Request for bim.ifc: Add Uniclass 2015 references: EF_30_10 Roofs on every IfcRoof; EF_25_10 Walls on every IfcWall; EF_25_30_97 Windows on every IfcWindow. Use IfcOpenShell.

First a look at what the model holds.

```python
import ifcopenshell

model = ifcopenshell.open("bim.ifc")
print(model.schema)
print("classifications:", [c.Name for c in model.by_type("IfcClassification")])
for ifc_class in ("IfcDoor", "IfcRoof", "IfcStair", "IfcWall", "IfcWindow"):
    print(ifc_class, len(model.by_type(ifc_class)))
```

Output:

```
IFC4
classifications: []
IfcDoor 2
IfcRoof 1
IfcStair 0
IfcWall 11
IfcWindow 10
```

```python
import ifcopenshell
import ifcopenshell.api.classification

model = ifcopenshell.open("bim.ifc")

system = ifcopenshell.api.classification.add_classification(model, classification="Uniclass 2015")

codes = {
    "IfcRoof": ("EF_30_10", "Roofs"),
    "IfcWall": ("EF_25_10", "Walls"),
    "IfcWindow": ("EF_25_30_97", "Windows"),
}
for ifc_class, (code, name) in codes.items():
    products = model.by_type(ifc_class)
    ifcopenshell.api.classification.add_reference(
        model, products=products, classification=system, identification=code, name=name
    )
    print(code, len(products))

model.write("bim_updated.ifc")
```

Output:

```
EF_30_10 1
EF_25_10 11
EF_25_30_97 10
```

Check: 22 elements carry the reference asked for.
